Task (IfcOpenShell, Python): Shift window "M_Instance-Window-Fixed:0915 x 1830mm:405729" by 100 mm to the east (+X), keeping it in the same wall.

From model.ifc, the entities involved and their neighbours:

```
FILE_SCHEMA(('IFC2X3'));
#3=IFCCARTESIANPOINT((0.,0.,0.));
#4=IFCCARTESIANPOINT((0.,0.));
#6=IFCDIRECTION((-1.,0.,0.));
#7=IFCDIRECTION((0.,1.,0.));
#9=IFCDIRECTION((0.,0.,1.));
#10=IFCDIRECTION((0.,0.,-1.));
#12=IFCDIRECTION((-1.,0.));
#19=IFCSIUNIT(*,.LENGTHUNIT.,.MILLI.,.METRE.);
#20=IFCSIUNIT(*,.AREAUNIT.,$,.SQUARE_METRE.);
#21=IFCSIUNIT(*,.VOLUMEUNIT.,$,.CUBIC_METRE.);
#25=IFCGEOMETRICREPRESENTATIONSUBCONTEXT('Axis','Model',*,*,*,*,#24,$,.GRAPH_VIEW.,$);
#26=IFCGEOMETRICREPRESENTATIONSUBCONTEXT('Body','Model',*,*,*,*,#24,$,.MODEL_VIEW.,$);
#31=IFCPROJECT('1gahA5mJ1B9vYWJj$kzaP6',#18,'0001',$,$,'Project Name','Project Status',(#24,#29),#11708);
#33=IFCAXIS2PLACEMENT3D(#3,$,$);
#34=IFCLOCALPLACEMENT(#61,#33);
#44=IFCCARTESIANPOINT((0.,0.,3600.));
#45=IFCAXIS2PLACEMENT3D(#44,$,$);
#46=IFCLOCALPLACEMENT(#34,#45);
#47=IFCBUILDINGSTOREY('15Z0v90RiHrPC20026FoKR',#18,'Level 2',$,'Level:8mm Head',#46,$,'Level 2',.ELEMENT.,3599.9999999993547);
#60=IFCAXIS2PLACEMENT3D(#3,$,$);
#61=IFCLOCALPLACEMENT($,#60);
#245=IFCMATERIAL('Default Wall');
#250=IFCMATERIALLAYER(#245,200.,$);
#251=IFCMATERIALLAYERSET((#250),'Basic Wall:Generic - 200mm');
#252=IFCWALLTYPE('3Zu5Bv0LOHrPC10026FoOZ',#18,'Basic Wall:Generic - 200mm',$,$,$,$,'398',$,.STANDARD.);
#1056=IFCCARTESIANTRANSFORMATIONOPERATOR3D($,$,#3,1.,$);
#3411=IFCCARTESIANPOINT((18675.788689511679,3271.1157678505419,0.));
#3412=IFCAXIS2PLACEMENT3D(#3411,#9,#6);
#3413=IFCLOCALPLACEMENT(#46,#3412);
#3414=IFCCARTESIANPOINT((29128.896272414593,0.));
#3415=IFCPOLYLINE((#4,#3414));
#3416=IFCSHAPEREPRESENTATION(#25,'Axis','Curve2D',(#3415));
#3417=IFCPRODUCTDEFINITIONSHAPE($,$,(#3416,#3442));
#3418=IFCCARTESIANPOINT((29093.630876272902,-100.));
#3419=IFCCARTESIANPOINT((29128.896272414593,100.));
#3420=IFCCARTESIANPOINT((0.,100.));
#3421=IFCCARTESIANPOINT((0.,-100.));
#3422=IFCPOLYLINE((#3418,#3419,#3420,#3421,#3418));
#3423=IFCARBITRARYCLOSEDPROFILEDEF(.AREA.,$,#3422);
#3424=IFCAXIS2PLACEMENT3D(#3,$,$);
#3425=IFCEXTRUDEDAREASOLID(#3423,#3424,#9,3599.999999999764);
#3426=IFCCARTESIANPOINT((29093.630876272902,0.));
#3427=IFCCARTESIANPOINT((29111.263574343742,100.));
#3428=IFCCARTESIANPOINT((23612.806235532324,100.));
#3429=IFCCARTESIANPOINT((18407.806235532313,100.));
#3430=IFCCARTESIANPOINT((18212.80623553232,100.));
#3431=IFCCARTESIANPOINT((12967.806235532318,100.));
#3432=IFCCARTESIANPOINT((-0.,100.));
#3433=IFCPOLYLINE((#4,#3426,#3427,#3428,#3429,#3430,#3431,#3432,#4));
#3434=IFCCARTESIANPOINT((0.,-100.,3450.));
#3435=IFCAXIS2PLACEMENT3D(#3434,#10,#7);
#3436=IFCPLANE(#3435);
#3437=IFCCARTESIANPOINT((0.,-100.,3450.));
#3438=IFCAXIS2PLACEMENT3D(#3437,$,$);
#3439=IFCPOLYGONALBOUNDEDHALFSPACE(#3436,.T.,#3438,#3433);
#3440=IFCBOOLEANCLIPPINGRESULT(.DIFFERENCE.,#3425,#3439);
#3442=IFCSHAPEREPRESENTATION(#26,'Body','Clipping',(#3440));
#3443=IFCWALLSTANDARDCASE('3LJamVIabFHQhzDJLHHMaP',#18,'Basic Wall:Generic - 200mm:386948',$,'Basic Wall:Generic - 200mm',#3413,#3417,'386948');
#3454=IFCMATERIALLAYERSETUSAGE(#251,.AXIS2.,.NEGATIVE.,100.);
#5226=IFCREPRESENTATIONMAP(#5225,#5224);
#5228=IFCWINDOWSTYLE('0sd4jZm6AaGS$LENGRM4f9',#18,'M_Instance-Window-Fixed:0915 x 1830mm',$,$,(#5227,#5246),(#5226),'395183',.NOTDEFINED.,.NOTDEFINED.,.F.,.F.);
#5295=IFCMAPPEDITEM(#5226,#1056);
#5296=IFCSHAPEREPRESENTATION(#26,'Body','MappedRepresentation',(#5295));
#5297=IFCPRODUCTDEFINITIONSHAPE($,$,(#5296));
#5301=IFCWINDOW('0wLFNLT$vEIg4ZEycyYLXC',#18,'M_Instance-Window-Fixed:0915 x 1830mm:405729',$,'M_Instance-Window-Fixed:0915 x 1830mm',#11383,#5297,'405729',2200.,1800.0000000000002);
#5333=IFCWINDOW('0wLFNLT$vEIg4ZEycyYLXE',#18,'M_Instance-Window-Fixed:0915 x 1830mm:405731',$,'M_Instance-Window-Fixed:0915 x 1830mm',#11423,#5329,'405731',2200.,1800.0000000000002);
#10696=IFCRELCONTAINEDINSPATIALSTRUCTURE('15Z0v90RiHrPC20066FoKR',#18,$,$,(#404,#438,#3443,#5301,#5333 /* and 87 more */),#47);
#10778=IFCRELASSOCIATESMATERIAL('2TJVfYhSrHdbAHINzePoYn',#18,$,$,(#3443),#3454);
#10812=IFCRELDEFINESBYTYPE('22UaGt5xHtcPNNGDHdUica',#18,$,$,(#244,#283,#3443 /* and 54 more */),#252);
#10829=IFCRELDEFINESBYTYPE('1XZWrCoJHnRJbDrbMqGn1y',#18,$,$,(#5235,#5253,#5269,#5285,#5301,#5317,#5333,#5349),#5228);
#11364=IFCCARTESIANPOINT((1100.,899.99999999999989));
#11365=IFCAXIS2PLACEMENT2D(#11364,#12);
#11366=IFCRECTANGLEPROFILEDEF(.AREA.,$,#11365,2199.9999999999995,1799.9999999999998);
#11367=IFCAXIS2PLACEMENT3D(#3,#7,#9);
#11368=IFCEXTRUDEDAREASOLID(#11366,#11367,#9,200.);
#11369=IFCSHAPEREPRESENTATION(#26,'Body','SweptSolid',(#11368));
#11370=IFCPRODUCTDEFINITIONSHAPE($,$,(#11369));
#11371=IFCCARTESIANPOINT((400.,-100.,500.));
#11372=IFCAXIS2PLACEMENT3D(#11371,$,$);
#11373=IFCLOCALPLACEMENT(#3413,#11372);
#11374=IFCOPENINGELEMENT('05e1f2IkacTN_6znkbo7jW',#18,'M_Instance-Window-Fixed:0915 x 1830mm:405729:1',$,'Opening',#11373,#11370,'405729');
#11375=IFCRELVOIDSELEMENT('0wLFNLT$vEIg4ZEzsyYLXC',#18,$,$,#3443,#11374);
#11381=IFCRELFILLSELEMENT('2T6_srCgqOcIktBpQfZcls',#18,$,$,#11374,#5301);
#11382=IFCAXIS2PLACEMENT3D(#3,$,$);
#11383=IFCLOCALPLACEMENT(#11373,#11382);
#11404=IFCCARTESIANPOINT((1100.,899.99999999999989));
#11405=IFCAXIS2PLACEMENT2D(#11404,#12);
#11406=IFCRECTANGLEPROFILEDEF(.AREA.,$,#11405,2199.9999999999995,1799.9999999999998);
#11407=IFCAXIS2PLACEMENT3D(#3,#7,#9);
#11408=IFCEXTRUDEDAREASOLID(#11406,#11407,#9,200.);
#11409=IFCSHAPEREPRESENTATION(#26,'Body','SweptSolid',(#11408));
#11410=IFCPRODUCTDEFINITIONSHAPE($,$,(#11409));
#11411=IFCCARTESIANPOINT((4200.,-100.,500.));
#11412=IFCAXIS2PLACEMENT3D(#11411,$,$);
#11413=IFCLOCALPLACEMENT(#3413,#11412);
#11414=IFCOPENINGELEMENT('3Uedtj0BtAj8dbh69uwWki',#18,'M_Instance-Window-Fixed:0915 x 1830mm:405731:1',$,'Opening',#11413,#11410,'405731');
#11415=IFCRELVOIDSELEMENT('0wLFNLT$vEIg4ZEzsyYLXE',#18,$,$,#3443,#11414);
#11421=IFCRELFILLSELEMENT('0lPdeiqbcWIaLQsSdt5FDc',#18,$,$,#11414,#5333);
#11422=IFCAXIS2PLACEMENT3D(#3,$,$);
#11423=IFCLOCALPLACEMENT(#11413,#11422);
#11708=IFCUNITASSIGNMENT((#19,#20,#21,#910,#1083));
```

```python
import ifcopenshell
import ifcopenshell.api.geometry
import ifcopenshell.util.placement

model = ifcopenshell.open("model.ifc")

window = model.by_guid("0wLFNLT$vEIg4ZEycyYLXC")
opening = window.FillsVoids[0].RelatingOpeningElement
wall = opening.VoidsElements[0].RelatingBuildingElement

wall_matrix = ifcopenshell.util.placement.get_local_placement(wall.ObjectPlacement)
shift = wall_matrix[:3, 0] * -100.0
before = ifcopenshell.util.placement.get_local_placement(window.ObjectPlacement)[:3, 3].copy()

# The window is placed relative to its opening, so it follows when the opening moves.
matrix = ifcopenshell.util.placement.get_local_placement(opening.ObjectPlacement)
matrix[:3, 3] += shift
ifcopenshell.api.geometry.edit_object_placement(
    model, product=opening, matrix=matrix, is_si=False, should_transform_children=True
)

after = ifcopenshell.util.placement.get_local_placement(window.ObjectPlacement)[:3, 3]
print("window moved by", (after - before).round(3) + 0.0)

model.write("model_edited.ifc")
```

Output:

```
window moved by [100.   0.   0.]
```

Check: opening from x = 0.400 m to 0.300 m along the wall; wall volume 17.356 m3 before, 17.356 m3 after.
